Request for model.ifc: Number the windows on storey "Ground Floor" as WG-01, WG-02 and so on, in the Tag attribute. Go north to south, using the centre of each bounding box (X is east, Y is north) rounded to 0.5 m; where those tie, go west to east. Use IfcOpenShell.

First a look at what the model holds.

```python
import ifcopenshell
import ifcopenshell.util.element
import ifcopenshell.util.placement

model = ifcopenshell.open("model.ifc")
print(model.schema)
storey = next(s for s in model.by_type("IfcBuildingStorey") if s.Name == "Ground Floor")
windows = [e for e in ifcopenshell.util.element.get_decomposition(storey) if e.is_a("IfcWindow")]
for e in sorted(windows, key=lambda e: e.id()):
    origin = ifcopenshell.util.placement.get_local_placement(e.ObjectPlacement)[:3, 3]
    print(e.id(), e.Tag, e.Name, origin.round(2) + 0.0, sep=" | ")
```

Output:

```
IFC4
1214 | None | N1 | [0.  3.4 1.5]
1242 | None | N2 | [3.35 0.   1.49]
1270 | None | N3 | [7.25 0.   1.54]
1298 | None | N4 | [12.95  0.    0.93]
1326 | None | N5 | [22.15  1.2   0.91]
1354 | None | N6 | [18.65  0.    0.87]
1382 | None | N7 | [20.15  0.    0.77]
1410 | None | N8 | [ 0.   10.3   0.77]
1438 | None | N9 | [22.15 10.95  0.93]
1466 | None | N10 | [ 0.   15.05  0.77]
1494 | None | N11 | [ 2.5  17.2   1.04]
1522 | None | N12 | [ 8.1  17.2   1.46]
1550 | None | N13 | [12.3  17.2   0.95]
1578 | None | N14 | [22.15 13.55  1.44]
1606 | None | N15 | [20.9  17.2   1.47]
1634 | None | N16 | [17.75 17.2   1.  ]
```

```python
import ifcopenshell
import ifcopenshell.geom
import ifcopenshell.util.element
import ifcopenshell.util.shape

model = ifcopenshell.open("model.ifc")
settings = ifcopenshell.geom.settings()
settings.set("use-world-coords", True)


def centre(element):
    shape = ifcopenshell.geom.create_shape(settings, element)
    return ifcopenshell.util.shape.get_bbox_centroid(shape.geometry)


storey = next(s for s in model.by_type("IfcBuildingStorey") if s.Name == "Ground Floor")
windows = [e for e in ifcopenshell.util.element.get_decomposition(storey) if e.is_a("IfcWindow")]

# Insertion points can sit at a corner or the storey origin, so sort by the geometry (in metres).
centres = {e: centre(e) for e in windows}
windows.sort(key=lambda e: (-round(centres[e][1] / 0.5), centres[e][0]))

for i, e in enumerate(windows, start=1):
    number = f"WG-{i:02d}"
    e.Tag = number
    print(e.id(), number)

model.write("model_v2.ifc")
```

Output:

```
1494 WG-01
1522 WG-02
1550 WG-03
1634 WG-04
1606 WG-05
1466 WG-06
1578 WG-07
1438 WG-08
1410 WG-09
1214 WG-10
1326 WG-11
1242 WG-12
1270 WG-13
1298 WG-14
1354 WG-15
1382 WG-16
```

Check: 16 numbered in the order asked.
